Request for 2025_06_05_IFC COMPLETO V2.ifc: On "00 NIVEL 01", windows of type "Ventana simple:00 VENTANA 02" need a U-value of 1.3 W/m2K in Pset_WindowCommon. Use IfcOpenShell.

First a look at what the model holds.

```python
import ifcopenshell
import ifcopenshell.util.element

model = ifcopenshell.open("2025_06_05_IFC COMPLETO V2.ifc")
print(model.schema)
storey = next(s for s in model.by_type("IfcBuildingStorey") if s.Name == "00 NIVEL 01")
windows = [e for e in ifcopenshell.util.element.get_decomposition(storey) if e.is_a("IfcWindow")]
seen = {}
for e in windows:
    element_type = ifcopenshell.util.element.get_type(e)
    key = (element_type.Name if element_type != e and element_type else None, ifcopenshell.util.element.get_pset(e, "Pset_WindowCommon", "ThermalTransmittance"))
    seen[key] = seen.get(key, 0) + 1
for (name, value), count in sorted(seen.items(), key=str):
    print(count, "x", name, "|", value)
```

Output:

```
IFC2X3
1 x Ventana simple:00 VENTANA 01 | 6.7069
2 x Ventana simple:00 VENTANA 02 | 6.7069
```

```python
import ifcopenshell
import ifcopenshell.api.pset
import ifcopenshell.util.element

model = ifcopenshell.open("2025_06_05_IFC COMPLETO V2.ifc")

storey = next(s for s in model.by_type("IfcBuildingStorey") if s.Name == "00 NIVEL 01")
windows = [e for e in ifcopenshell.util.element.get_decomposition(storey) if e.is_a("IfcWindow")]

count = 0
for e in windows:
    element_type = ifcopenshell.util.element.get_type(e)
    if element_type in (None, e) or element_type.Name != "Ventana simple:00 VENTANA 02":
        continue
    # add_pset returns the element's existing set when there is one.
    pset = ifcopenshell.api.pset.add_pset(model, product=e, name="Pset_WindowCommon")
    ifcopenshell.api.pset.edit_pset(model, pset=pset, properties={"ThermalTransmittance": 1.3})
    count += 1

print(count, "windows updated")

model.write("2025_06_05_IFC COMPLETO V2_updated.ifc")
```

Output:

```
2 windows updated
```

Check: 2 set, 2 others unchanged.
